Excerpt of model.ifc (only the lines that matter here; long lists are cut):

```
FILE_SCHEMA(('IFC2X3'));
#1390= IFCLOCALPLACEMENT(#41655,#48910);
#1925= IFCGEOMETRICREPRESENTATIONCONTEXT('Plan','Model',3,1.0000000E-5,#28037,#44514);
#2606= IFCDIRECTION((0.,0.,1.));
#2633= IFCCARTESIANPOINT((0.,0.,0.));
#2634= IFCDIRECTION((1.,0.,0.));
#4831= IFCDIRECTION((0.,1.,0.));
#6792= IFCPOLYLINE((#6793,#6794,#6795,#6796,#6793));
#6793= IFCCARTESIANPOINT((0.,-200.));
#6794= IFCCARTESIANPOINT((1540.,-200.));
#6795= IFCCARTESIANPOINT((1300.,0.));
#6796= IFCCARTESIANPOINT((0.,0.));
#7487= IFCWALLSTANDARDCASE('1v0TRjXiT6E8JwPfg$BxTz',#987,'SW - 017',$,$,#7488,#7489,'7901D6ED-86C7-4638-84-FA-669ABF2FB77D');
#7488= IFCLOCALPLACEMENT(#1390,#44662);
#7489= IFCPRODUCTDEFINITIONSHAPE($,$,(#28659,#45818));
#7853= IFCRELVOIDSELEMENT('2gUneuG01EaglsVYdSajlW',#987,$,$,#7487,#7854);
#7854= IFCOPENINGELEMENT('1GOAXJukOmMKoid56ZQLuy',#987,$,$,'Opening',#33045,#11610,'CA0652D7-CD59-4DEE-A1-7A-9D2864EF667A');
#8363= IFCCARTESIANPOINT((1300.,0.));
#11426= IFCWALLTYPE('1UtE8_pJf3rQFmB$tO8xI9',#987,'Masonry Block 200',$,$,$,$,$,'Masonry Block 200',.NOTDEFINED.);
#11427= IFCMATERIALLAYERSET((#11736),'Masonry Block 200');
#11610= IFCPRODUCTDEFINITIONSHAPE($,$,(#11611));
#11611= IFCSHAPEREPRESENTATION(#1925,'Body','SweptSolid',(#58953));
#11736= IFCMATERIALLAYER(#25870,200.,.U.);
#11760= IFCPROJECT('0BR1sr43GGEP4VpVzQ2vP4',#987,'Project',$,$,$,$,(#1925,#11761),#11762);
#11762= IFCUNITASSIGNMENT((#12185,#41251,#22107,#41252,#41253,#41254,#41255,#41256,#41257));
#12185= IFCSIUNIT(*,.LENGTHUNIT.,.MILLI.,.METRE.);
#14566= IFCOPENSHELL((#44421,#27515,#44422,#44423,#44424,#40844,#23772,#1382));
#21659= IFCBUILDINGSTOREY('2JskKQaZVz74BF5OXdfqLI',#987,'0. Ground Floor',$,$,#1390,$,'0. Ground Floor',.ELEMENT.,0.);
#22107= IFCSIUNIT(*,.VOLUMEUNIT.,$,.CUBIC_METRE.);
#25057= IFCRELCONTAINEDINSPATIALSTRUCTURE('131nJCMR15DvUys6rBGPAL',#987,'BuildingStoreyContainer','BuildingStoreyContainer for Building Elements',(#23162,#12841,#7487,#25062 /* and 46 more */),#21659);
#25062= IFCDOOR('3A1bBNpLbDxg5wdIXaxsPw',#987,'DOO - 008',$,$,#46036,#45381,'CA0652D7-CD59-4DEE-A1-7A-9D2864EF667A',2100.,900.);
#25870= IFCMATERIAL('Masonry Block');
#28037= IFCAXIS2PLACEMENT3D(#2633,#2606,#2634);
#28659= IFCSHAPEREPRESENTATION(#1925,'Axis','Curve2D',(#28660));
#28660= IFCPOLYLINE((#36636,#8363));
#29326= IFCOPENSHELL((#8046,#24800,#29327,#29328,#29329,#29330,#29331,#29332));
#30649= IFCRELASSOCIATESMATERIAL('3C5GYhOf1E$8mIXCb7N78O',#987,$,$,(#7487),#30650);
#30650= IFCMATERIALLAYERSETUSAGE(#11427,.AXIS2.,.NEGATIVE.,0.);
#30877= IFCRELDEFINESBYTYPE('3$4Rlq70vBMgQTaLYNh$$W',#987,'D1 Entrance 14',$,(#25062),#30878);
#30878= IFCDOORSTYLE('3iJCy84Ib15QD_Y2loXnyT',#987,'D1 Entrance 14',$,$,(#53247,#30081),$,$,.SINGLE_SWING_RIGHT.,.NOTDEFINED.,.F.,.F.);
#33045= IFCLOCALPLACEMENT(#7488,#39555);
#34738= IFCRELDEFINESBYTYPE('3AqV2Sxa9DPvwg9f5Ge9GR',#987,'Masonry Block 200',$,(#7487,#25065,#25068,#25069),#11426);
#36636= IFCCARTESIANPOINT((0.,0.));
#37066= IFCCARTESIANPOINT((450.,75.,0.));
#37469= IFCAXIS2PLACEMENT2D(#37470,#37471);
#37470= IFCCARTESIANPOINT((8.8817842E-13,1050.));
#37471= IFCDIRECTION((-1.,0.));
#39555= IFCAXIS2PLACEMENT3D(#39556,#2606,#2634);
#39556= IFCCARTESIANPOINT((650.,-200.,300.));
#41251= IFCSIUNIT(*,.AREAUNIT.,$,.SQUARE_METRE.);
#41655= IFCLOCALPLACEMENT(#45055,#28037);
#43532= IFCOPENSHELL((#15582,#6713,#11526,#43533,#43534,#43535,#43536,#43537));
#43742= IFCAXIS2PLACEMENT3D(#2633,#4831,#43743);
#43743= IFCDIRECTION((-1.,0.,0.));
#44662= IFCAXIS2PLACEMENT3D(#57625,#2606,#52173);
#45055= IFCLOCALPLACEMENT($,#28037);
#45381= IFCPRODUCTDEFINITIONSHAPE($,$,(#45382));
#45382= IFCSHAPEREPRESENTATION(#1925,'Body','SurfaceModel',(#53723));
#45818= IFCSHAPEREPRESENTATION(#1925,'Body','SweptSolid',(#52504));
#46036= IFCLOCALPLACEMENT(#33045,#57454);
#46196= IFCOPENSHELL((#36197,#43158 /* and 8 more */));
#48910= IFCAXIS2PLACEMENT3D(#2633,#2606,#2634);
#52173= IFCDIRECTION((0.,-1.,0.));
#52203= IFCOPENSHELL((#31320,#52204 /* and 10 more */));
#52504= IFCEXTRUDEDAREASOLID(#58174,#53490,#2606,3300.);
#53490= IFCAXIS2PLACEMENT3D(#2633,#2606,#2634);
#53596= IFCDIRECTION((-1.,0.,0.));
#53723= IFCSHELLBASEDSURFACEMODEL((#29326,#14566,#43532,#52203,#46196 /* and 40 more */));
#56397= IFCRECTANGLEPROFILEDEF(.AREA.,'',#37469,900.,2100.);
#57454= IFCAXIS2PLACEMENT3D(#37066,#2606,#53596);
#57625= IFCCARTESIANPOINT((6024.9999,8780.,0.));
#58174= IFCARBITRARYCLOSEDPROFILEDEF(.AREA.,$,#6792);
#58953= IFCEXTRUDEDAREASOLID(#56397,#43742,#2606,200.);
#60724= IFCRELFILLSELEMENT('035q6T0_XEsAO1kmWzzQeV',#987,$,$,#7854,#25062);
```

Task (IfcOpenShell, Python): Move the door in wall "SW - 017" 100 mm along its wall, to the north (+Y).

```python
import ifcopenshell
import ifcopenshell.api.geometry
import ifcopenshell.util.placement
import ifcopenshell.util.unit

model = ifcopenshell.open("model.ifc")
unit_scale = ifcopenshell.util.unit.calculate_unit_scale(model)

door = model.by_guid("3A1bBNpLbDxg5wdIXaxsPw")
opening = door.FillsVoids[0].RelatingOpeningElement
wall = opening.VoidsElements[0].RelatingBuildingElement

wall_matrix = ifcopenshell.util.placement.get_local_placement(wall.ObjectPlacement)
shift = wall_matrix[:3, 0] * -0.1 / unit_scale
before = ifcopenshell.util.placement.get_local_placement(door.ObjectPlacement)[:3, 3].copy()

# The door is placed relative to its opening, so it follows when the opening moves.
matrix = ifcopenshell.util.placement.get_local_placement(opening.ObjectPlacement)
matrix[:3, 3] += shift
ifcopenshell.api.geometry.edit_object_placement(
    model, product=opening, matrix=matrix, is_si=False, should_transform_children=True
)

after = ifcopenshell.util.placement.get_local_placement(door.ObjectPlacement)[:3, 3]
print("door moved by", (after - before).round(3) + 0.0)

model.write("model-out.ifc")
```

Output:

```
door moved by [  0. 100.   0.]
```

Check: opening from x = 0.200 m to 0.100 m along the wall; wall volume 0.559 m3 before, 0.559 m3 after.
